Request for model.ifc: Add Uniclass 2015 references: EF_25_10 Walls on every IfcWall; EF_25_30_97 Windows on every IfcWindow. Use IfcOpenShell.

First a look at what the model holds.

```python
import ifcopenshell

model = ifcopenshell.open("model.ifc")
print(model.schema)
print("classifications:", [c.Name for c in model.by_type("IfcClassification")])
for ifc_class in ("IfcDoor", "IfcRoof", "IfcStair", "IfcWall", "IfcWindow"):
    print(ifc_class, len(model.by_type(ifc_class)))
```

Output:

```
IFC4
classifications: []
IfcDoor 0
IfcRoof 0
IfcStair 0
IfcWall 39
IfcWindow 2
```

```python
import ifcopenshell
import ifcopenshell.api.classification

model = ifcopenshell.open("model.ifc")

system = ifcopenshell.api.classification.add_classification(model, classification="Uniclass 2015")

codes = {
    "IfcWall": ("EF_25_10", "Walls"),
    "IfcWindow": ("EF_25_30_97", "Windows"),
}
for ifc_class, (code, name) in codes.items():
    products = model.by_type(ifc_class)
    ifcopenshell.api.classification.add_reference(
        model, products=products, classification=system, identification=code, name=name
    )
    print(code, len(products))

model.write("model_updated.ifc")
```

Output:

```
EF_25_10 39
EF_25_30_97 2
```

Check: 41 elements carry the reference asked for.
